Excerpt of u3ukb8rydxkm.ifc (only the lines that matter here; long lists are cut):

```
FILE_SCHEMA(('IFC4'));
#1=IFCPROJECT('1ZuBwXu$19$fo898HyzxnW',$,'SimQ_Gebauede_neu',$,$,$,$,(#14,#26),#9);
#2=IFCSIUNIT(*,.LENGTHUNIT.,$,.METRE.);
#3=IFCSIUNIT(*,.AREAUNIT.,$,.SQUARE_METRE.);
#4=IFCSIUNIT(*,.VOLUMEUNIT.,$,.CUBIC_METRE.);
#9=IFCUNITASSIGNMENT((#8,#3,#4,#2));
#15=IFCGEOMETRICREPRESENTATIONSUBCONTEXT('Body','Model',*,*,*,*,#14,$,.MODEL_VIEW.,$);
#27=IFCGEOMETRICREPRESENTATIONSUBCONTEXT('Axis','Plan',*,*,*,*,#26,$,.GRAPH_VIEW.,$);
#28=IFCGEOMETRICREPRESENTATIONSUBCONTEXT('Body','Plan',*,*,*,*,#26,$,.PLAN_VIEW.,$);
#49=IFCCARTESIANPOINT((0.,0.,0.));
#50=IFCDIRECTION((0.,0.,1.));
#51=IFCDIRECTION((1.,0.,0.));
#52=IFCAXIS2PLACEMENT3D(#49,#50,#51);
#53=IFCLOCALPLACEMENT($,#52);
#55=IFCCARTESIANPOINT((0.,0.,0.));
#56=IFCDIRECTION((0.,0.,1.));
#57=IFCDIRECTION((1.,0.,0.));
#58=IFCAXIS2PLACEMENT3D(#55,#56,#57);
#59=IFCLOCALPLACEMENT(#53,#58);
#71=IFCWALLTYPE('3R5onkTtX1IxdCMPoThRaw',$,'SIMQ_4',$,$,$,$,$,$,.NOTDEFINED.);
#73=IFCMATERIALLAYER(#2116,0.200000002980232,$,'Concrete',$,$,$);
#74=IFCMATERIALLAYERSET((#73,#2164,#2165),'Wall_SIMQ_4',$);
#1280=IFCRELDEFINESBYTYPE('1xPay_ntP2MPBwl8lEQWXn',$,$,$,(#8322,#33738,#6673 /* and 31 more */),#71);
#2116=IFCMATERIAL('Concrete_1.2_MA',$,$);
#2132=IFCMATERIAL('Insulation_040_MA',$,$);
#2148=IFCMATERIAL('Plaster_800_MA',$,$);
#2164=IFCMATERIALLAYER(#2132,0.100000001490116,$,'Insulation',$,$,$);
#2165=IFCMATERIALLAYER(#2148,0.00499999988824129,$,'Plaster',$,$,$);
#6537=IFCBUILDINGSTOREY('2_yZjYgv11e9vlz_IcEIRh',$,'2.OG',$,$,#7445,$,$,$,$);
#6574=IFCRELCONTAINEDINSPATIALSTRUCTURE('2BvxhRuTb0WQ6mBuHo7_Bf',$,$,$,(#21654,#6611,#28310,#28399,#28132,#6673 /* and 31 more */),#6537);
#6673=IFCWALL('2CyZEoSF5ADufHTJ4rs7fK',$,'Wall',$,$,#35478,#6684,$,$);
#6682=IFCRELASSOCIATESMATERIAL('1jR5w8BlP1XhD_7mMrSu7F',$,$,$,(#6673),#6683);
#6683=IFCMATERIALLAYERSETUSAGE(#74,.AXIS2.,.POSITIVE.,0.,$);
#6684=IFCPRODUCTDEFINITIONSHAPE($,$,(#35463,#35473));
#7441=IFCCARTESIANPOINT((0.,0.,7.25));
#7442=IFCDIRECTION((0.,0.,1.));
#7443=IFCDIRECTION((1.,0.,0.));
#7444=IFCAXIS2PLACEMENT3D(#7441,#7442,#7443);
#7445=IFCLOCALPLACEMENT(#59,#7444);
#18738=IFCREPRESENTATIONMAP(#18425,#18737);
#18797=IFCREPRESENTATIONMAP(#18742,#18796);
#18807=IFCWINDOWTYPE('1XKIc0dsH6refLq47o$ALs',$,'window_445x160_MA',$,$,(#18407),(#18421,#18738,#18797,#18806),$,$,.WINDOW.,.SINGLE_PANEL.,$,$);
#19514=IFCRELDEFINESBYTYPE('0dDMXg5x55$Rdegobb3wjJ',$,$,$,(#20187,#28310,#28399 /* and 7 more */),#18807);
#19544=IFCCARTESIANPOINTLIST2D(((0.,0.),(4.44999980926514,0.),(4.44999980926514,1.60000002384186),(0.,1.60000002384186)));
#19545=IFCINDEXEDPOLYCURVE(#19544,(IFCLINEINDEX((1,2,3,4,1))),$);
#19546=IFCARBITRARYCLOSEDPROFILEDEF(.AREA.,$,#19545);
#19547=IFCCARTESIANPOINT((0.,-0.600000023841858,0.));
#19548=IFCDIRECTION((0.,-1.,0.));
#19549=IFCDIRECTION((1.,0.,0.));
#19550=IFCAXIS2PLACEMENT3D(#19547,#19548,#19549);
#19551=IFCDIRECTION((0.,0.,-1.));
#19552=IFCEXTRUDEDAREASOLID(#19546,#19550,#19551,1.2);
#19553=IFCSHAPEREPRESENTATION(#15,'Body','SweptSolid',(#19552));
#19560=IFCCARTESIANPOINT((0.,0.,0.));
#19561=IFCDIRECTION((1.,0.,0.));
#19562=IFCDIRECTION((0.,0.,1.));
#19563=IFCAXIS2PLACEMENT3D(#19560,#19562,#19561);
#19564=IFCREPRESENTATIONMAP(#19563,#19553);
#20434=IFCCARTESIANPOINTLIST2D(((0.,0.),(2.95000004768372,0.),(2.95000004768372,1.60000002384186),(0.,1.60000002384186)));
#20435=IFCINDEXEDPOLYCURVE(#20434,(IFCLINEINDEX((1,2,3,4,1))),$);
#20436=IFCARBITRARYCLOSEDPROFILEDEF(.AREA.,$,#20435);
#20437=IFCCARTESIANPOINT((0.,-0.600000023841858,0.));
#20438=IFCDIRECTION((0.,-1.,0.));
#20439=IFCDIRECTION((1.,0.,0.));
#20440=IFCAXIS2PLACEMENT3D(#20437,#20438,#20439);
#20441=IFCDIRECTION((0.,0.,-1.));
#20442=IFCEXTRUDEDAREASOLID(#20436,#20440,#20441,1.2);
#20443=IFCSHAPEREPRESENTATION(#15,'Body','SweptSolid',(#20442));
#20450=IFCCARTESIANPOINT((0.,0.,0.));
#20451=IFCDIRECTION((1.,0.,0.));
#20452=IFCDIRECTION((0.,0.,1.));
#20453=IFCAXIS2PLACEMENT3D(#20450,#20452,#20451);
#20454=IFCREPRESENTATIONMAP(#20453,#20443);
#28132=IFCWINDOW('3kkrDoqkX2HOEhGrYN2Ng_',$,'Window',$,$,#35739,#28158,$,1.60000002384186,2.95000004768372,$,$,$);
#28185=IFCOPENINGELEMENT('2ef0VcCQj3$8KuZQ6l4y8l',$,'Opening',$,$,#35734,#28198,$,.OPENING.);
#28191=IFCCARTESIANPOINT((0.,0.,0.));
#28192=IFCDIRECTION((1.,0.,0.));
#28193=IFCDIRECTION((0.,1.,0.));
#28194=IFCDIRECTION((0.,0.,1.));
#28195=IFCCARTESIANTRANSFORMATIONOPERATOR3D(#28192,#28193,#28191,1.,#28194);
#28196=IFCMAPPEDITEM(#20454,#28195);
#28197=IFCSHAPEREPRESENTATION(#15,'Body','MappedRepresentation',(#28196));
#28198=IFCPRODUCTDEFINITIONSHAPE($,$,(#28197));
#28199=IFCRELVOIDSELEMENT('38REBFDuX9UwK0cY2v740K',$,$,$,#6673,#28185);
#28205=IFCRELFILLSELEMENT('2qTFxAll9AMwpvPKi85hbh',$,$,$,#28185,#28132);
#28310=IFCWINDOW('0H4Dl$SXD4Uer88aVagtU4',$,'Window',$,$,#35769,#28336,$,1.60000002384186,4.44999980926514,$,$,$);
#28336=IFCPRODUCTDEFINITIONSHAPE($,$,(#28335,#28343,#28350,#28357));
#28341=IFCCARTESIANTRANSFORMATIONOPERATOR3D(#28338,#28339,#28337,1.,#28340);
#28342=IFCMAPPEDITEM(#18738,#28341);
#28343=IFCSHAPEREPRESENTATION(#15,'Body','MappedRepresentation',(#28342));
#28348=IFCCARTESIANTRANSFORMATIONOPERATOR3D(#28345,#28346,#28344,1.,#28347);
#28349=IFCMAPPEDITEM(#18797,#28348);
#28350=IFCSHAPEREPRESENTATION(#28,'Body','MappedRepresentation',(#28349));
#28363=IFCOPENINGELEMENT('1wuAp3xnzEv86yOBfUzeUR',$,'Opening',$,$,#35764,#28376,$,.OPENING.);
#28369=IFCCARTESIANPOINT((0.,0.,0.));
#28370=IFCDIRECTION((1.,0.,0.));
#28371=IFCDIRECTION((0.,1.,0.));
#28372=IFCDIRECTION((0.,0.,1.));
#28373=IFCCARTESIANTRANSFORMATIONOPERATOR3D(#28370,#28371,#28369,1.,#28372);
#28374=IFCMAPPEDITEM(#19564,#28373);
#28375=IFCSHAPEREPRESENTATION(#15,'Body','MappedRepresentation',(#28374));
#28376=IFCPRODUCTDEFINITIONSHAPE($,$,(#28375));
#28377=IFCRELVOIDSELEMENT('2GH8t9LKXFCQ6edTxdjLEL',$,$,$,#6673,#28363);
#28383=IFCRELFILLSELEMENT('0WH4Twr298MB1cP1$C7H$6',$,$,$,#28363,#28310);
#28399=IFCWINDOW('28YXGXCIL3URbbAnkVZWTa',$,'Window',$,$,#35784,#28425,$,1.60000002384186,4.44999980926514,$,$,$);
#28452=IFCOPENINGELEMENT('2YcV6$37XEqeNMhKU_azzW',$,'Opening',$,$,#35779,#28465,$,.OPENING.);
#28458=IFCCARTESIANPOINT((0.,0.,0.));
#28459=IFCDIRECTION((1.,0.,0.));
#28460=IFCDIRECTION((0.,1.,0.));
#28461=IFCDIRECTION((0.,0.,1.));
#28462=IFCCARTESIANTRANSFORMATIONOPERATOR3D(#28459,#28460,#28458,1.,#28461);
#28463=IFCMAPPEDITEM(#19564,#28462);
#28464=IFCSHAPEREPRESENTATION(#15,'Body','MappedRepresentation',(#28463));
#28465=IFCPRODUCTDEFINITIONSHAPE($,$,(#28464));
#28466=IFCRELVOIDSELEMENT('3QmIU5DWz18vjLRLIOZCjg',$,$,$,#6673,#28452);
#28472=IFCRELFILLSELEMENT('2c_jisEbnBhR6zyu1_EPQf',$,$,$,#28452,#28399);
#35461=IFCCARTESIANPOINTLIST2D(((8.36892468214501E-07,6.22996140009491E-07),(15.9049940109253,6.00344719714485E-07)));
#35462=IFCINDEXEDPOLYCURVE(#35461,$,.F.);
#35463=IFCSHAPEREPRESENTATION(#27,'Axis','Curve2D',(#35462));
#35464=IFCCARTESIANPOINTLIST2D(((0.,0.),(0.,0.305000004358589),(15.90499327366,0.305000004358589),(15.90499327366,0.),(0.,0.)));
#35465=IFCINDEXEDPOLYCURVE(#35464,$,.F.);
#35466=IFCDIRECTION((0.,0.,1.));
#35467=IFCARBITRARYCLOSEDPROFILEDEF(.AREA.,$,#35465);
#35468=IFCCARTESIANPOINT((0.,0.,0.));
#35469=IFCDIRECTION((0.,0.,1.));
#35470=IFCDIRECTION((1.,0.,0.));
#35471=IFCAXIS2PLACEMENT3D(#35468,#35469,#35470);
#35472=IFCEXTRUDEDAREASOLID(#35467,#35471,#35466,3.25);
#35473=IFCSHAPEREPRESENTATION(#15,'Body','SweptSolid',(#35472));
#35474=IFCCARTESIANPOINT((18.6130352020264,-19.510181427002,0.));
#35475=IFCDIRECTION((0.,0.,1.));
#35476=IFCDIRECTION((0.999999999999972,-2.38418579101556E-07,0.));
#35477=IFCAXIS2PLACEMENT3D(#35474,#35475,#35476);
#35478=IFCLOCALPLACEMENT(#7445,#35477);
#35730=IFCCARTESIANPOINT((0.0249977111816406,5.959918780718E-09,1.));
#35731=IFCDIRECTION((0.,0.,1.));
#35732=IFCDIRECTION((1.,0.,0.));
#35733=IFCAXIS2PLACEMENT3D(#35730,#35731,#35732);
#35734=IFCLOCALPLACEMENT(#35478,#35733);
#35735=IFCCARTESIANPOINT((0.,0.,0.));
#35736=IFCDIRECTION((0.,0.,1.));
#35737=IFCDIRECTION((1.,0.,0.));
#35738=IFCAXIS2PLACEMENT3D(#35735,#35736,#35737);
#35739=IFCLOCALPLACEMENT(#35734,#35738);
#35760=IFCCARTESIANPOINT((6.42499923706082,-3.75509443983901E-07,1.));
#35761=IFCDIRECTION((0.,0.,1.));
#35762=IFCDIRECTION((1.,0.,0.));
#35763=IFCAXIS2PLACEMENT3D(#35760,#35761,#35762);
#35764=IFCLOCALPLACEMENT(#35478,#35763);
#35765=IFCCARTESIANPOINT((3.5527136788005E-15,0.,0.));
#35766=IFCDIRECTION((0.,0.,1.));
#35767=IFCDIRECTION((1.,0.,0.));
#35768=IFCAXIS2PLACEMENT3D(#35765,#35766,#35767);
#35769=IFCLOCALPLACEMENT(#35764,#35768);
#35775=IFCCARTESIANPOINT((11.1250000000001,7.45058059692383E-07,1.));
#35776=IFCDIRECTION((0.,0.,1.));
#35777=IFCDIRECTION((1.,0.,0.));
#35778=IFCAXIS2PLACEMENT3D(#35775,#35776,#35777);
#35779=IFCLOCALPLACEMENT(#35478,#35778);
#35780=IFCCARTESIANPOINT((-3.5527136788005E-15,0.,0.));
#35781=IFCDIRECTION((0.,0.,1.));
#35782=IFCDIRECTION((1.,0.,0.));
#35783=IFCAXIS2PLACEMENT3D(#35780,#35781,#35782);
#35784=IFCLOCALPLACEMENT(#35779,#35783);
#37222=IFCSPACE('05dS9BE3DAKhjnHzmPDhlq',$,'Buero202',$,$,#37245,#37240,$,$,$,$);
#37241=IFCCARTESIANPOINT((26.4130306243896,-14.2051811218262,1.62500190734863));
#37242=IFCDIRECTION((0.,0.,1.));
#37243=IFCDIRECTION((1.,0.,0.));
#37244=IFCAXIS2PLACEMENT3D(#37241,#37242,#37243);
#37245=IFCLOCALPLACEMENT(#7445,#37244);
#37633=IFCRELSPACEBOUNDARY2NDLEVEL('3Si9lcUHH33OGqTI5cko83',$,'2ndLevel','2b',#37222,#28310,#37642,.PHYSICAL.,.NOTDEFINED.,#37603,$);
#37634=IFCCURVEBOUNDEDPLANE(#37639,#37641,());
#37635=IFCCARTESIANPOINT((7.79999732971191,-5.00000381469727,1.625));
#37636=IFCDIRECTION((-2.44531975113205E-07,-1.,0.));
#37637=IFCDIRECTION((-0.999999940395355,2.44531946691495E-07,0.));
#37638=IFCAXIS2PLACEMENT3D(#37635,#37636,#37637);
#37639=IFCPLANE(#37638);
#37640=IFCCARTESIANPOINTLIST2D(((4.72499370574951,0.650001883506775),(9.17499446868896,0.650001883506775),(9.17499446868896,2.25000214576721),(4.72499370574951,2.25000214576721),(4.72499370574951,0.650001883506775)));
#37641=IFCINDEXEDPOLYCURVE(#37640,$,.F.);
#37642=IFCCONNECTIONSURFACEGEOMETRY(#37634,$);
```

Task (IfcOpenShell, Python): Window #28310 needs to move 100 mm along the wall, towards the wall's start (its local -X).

```python
import numpy as np
import ifcopenshell
import ifcopenshell.api.geometry
import ifcopenshell.util.placement
import ifcopenshell.util.unit

model = ifcopenshell.open("u3ukb8rydxkm.ifc")
unit_scale = ifcopenshell.util.unit.calculate_unit_scale(model)

window = model.by_id(28310)
opening = window.FillsVoids[0].RelatingOpeningElement
wall = opening.VoidsElements[0].RelatingBuildingElement

wall_matrix = ifcopenshell.util.placement.get_local_placement(wall.ObjectPlacement)
shift = wall_matrix[:3, 0] * -0.1 / unit_scale
before = ifcopenshell.util.placement.get_local_placement(window.ObjectPlacement)[:3, 3].copy()

# The window is placed relative to its opening, so it follows when the opening moves.
matrix = ifcopenshell.util.placement.get_local_placement(opening.ObjectPlacement)
matrix[:3, 3] += shift
ifcopenshell.api.geometry.edit_object_placement(
    model, product=opening, matrix=matrix, is_si=False, should_transform_children=True
)

# Space boundary surfaces are stored in each space's coordinates; move them too.
for rel in window.ProvidesBoundaries:
    if not rel.ConnectionGeometry:
        continue
    surface = rel.ConnectionGeometry.SurfaceOnRelatingElement.BasisSurface
    space_matrix = ifcopenshell.util.placement.get_local_placement(rel.RelatingSpace.ObjectPlacement)
    point = np.array(surface.Position.Location.Coordinates) + space_matrix[:3, :3].T @ shift
    surface.Position = model.createIfcAxis2Placement3D(
        model.createIfcCartesianPoint(point.tolist()), surface.Position.Axis, surface.Position.RefDirection
    )

after = ifcopenshell.util.placement.get_local_placement(window.ObjectPlacement)[:3, 3]
print("window moved by", (after - before).round(3) + 0.0)

model.write("u3ukb8rydxkm_v2.ifc")
```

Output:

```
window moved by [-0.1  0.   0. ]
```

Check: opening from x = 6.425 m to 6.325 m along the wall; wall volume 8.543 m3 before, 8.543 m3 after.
